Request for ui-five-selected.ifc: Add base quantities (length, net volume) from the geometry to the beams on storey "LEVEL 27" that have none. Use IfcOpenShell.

First a look at what the model holds.

```python
import ifcopenshell
import ifcopenshell.util.element
import ifcopenshell.util.unit

model = ifcopenshell.open("ui-five-selected.ifc")
print(model.schema)
for unit_type in ("LENGTHUNIT", "AREAUNIT", "VOLUMEUNIT"):
    print(unit_type, ifcopenshell.util.unit.calculate_unit_scale(model, unit_type))
storey = next(s for s in model.by_type("IfcBuildingStorey") if s.Name == "LEVEL 27")
beams = [e for e in ifcopenshell.util.element.get_decomposition(storey) if e.is_a("IfcBeam")]
for e in sorted(beams, key=lambda e: e.id()):
    print(e.id(), e.is_a(), e.Name, list(ifcopenshell.util.element.get_psets(e, qtos_only=True)), sep=" | ")
```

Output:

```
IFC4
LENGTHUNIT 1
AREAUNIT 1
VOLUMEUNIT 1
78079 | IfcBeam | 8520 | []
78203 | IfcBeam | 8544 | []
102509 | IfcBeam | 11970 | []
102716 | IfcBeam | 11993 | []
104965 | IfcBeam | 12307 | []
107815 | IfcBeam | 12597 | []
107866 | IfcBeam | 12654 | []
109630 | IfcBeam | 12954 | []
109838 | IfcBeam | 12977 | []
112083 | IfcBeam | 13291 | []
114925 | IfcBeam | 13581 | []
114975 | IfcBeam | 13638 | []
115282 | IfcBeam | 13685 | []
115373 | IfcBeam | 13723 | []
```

```python
import ifcopenshell
import ifcopenshell.api.pset
import ifcopenshell.geom
import ifcopenshell.util.element
import ifcopenshell.util.shape
import ifcopenshell.util.unit

model = ifcopenshell.open("ui-five-selected.ifc")
unit_scale = ifcopenshell.util.unit.calculate_unit_scale(model)
volume_scale = ifcopenshell.util.unit.calculate_unit_scale(model, "VOLUMEUNIT")
settings = ifcopenshell.geom.settings()

storey = next(s for s in model.by_type("IfcBuildingStorey") if s.Name == "LEVEL 27")
beams = [e for e in ifcopenshell.util.element.get_decomposition(storey) if e.is_a("IfcBeam")]

for e in sorted(beams, key=lambda e: e.id()):
    if ifcopenshell.util.element.get_psets(e, qtos_only=True, should_inherit=False):
        continue
    # Geometry comes back in metres, in the element's own axes.
    shape = ifcopenshell.geom.create_shape(settings, e)
    values = {
        "Length": ifcopenshell.util.shape.get_max_xyz(shape.geometry) / unit_scale,
        "NetVolume": ifcopenshell.util.shape.get_volume(shape.geometry) / volume_scale,
    }
    qto = ifcopenshell.api.pset.add_qto(model, product=e, name="Qto_BeamBaseQuantities")
    ifcopenshell.api.pset.edit_qto(model, qto=qto, properties=values)
    print(e.id(), {k: round(v, 3) for k, v in values.items()})

model.write("ui-five-selected_edited.ifc")
```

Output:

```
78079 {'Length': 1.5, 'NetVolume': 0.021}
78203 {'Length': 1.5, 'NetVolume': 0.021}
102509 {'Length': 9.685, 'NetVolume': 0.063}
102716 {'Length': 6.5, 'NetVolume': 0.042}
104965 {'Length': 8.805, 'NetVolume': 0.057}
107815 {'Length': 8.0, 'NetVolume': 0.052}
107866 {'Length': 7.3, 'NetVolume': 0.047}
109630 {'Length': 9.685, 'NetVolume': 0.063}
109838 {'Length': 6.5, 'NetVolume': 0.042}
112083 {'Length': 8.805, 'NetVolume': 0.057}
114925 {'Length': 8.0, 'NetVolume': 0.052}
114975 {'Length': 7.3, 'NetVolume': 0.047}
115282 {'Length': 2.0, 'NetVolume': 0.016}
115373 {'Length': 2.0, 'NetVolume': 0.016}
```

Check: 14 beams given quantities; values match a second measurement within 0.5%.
